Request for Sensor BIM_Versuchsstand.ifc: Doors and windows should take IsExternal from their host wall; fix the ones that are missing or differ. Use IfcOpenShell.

First a look at what the model holds.

```python
import ifcopenshell
import ifcopenshell.util.element

model = ifcopenshell.open("Sensor BIM_Versuchsstand.ifc")
print(model.schema)
seen = {}
for e in model.by_type("IfcDoor") + model.by_type("IfcWindow"):
    if not e.FillsVoids:
        continue
    host = e.FillsVoids[0].RelatingOpeningElement.VoidsElements[0].RelatingBuildingElement
    own = ifcopenshell.util.element.get_pset(e, f"Pset_{e.is_a()[3:].removesuffix('StandardCase')}Common", "IsExternal")
    wall = ifcopenshell.util.element.get_pset(host, "Pset_WallCommon", "IsExternal")
    seen[e.is_a(), own, wall] = seen.get((e.is_a(), own, wall), 0) + 1
for (cls, own, wall), count in sorted(seen.items(), key=str):
    print(count, cls, "IsExternal:", own, "| host wall:", wall)
```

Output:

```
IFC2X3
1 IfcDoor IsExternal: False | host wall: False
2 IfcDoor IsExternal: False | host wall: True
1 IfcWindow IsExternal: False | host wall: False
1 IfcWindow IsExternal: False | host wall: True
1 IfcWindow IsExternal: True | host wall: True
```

```python
import ifcopenshell
import ifcopenshell.api.pset
import ifcopenshell.util.element

model = ifcopenshell.open("Sensor BIM_Versuchsstand.ifc")

count = 0
for ifc_class, pset_name in (("IfcDoor", "Pset_DoorCommon"), ("IfcWindow", "Pset_WindowCommon")):
    for e in model.by_type(ifc_class):
        if not e.FillsVoids:
            continue
        host = e.FillsVoids[0].RelatingOpeningElement.VoidsElements[0].RelatingBuildingElement
        external = ifcopenshell.util.element.get_pset(host, "Pset_WallCommon", "IsExternal")
        if external is None or ifcopenshell.util.element.get_pset(e, pset_name, "IsExternal") == external:
            continue
        pset = ifcopenshell.api.pset.add_pset(model, product=e, name=pset_name)
        ifcopenshell.api.pset.edit_pset(model, pset=pset, properties={"IsExternal": external})
        count += 1

print(count, "updated")

model.write("Sensor BIM_Versuchsstand_rev.ifc")
```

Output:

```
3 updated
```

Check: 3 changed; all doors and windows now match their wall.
